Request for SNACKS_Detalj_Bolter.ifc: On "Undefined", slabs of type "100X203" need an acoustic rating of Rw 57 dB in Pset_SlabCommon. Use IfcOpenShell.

First a look at what the model holds.

```python
import ifcopenshell
import ifcopenshell.util.element

model = ifcopenshell.open("SNACKS_Detalj_Bolter.ifc")
print(model.schema)
storey = next(s for s in model.by_type("IfcBuildingStorey") if s.Name == "Undefined")
slabs = [e for e in ifcopenshell.util.element.get_decomposition(storey) if e.is_a("IfcSlab")]
seen = {}
for e in slabs:
    element_type = ifcopenshell.util.element.get_type(e)
    key = (element_type.Name if element_type != e and element_type else None, ifcopenshell.util.element.get_pset(e, "Pset_SlabCommon", "AcousticRating"))
    seen[key] = seen.get(key, 0) + 1
for (name, value), count in sorted(seen.items(), key=str):
    print(count, "x", name, "|", value)
```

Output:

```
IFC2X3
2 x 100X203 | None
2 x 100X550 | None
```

```python
import ifcopenshell
import ifcopenshell.api.pset
import ifcopenshell.util.element

model = ifcopenshell.open("SNACKS_Detalj_Bolter.ifc")

storey = next(s for s in model.by_type("IfcBuildingStorey") if s.Name == "Undefined")
slabs = [e for e in ifcopenshell.util.element.get_decomposition(storey) if e.is_a("IfcSlab")]

count = 0
for e in slabs:
    element_type = ifcopenshell.util.element.get_type(e)
    if element_type in (None, e) or element_type.Name != "100X203":
        continue
    # add_pset returns the element's existing set when there is one.
    pset = ifcopenshell.api.pset.add_pset(model, product=e, name="Pset_SlabCommon")
    ifcopenshell.api.pset.edit_pset(model, pset=pset, properties={"AcousticRating": "Rw 57 dB"})
    count += 1

print(count, "slabs updated")

model.write("SNACKS_Detalj_Bolter_edited.ifc")
```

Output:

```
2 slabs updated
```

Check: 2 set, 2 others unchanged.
